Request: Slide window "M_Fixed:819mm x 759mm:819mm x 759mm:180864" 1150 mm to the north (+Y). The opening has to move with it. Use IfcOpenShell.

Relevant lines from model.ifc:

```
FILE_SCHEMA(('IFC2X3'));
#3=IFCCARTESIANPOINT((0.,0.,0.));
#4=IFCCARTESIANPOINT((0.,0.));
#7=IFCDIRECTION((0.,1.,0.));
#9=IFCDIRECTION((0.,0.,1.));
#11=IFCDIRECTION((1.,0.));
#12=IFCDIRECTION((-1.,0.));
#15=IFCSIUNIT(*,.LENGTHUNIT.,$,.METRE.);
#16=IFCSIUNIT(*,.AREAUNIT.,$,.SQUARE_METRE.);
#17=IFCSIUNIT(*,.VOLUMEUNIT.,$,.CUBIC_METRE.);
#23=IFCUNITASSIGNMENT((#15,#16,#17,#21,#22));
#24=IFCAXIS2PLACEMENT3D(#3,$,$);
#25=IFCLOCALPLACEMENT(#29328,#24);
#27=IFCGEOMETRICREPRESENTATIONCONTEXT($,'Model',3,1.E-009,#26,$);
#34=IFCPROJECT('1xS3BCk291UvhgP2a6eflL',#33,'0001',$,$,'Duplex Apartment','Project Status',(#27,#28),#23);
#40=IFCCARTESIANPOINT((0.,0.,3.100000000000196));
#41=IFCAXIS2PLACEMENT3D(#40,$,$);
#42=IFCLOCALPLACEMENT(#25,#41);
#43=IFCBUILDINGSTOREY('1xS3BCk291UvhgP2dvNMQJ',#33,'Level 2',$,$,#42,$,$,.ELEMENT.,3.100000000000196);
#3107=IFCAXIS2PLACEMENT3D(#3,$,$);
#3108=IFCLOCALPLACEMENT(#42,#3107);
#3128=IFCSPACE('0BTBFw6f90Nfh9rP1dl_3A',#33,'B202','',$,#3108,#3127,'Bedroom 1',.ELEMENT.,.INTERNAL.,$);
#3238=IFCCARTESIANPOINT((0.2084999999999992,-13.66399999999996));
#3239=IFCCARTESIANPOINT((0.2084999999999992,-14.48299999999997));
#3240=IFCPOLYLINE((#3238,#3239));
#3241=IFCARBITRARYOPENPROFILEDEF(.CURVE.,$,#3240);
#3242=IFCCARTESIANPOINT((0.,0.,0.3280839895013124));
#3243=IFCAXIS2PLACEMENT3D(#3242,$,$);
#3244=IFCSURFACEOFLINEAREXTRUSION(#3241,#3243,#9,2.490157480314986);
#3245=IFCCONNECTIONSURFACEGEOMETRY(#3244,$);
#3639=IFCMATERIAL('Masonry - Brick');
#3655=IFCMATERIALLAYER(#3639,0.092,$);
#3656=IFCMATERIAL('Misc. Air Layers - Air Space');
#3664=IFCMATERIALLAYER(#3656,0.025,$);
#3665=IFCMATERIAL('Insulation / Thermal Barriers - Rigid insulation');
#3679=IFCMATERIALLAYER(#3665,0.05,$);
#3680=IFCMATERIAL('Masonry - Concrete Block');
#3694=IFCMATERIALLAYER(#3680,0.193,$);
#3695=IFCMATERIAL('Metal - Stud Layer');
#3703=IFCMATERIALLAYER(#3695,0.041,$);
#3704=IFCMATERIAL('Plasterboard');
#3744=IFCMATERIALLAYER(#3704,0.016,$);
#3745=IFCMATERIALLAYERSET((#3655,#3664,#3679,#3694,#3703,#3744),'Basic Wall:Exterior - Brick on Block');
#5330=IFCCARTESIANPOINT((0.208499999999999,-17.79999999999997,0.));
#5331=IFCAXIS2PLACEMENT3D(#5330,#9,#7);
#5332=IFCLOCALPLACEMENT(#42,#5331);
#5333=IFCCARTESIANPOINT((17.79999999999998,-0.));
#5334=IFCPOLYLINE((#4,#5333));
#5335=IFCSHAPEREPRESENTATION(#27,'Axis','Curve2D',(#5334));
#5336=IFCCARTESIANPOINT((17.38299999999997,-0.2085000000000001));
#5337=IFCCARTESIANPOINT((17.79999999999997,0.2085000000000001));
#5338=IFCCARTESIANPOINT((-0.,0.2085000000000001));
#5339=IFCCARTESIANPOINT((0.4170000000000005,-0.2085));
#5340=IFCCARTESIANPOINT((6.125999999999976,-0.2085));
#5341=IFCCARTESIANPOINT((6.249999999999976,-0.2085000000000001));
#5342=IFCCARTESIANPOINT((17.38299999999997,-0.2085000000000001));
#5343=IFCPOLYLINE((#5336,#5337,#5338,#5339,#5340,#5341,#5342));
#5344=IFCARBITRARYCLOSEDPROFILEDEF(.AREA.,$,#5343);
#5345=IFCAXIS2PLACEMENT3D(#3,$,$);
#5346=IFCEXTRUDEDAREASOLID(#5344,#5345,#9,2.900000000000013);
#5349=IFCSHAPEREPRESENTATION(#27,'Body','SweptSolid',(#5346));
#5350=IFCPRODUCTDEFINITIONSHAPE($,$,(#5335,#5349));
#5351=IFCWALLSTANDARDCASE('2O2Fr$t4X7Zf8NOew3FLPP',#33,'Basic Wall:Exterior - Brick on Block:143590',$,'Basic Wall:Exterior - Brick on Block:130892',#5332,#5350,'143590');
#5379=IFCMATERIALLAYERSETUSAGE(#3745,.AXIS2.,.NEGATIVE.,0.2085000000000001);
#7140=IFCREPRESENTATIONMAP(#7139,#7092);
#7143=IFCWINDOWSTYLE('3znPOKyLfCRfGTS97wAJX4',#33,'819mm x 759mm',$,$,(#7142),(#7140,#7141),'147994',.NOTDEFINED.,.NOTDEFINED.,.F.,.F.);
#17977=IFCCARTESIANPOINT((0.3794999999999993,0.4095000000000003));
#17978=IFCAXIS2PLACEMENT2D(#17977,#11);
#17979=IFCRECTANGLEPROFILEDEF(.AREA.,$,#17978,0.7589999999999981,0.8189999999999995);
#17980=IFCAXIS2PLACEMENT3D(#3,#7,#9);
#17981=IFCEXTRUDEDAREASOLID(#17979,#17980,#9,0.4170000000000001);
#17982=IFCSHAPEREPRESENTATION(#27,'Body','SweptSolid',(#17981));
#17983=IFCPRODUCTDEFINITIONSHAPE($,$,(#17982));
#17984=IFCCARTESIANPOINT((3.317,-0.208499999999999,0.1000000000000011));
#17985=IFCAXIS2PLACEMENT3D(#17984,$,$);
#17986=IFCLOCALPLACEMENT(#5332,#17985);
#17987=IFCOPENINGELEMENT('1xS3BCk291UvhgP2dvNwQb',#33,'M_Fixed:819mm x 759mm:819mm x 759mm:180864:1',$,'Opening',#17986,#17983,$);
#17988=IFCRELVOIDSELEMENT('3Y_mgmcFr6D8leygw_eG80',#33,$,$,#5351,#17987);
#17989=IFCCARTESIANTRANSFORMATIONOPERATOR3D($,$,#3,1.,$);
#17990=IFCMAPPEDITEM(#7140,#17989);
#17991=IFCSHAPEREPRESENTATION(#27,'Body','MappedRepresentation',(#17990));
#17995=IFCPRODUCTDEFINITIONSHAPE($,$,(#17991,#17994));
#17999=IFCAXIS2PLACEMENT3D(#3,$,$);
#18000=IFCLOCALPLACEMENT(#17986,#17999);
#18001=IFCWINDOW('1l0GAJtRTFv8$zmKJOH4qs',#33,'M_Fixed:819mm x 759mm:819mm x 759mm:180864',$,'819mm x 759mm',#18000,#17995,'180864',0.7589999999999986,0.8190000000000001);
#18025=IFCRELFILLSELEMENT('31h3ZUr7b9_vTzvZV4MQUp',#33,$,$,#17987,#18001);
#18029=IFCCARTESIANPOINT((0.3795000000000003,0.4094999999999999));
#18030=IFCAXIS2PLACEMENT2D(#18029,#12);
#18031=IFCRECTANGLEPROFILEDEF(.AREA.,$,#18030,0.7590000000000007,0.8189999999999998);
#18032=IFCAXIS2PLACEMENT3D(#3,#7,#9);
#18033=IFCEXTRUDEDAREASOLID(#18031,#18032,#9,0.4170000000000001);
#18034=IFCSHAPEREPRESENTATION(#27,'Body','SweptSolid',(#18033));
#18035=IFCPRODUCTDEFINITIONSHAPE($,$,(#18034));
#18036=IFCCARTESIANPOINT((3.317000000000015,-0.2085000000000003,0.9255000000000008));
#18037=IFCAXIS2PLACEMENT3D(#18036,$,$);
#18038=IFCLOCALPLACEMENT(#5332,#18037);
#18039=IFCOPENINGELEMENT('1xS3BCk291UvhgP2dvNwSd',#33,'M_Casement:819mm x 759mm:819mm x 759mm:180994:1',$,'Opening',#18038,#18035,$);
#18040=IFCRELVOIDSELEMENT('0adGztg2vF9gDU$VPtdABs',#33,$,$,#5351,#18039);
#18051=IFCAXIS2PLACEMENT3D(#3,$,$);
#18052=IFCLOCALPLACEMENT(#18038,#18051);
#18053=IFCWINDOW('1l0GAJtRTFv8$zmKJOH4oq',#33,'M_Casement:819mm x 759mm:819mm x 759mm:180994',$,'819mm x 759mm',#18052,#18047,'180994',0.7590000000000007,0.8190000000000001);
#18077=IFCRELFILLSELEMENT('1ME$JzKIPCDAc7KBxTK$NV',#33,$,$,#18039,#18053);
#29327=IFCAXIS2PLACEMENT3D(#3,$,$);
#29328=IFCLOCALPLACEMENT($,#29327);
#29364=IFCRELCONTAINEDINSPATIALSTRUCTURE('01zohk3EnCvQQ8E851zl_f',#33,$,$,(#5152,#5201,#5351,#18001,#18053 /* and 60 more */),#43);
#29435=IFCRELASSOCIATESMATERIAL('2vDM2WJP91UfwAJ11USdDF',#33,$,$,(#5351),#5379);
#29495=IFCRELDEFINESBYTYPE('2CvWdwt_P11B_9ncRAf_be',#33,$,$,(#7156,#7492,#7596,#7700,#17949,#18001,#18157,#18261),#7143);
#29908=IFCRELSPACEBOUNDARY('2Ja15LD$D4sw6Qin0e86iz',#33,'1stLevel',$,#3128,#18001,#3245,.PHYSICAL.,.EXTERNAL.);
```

```python
import numpy as np
import ifcopenshell
import ifcopenshell.api.geometry
import ifcopenshell.util.placement

model = ifcopenshell.open("model.ifc")

window = model.by_id(18001)
opening = window.FillsVoids[0].RelatingOpeningElement
wall = opening.VoidsElements[0].RelatingBuildingElement

wall_matrix = ifcopenshell.util.placement.get_local_placement(wall.ObjectPlacement)
shift = wall_matrix[:3, 0] * 1.15
before = ifcopenshell.util.placement.get_local_placement(window.ObjectPlacement)[:3, 3].copy()

# The window is placed relative to its opening, so it follows when the opening moves.
matrix = ifcopenshell.util.placement.get_local_placement(opening.ObjectPlacement)
matrix[:3, 3] += shift
ifcopenshell.api.geometry.edit_object_placement(
    model, product=opening, matrix=matrix, is_si=False, should_transform_children=True
)

# Space boundary surfaces are stored in each space's coordinates; move them too.
for rel in window.ProvidesBoundaries:
    if not rel.ConnectionGeometry:
        continue
    surface = rel.ConnectionGeometry.SurfaceOnRelatingElement
    space_matrix = ifcopenshell.util.placement.get_local_placement(rel.RelatingSpace.ObjectPlacement)
    point = np.array(surface.Position.Location.Coordinates) + space_matrix[:3, :3].T @ shift
    surface.Position = model.createIfcAxis2Placement3D(
        model.createIfcCartesianPoint(point.tolist()), surface.Position.Axis, surface.Position.RefDirection
    )

after = ifcopenshell.util.placement.get_local_placement(window.ObjectPlacement)[:3, 3]
print("window moved by", (after - before).round(3) + 0.0)

model.write("model_updated.ifc")
```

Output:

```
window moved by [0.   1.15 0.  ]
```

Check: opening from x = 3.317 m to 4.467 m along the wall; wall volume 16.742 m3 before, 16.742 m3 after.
